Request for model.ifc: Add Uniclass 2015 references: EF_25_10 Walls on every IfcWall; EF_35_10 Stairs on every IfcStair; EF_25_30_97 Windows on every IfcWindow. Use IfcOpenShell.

First a look at what the model holds.

```python
import ifcopenshell

model = ifcopenshell.open("model.ifc")
print(model.schema)
print("classifications:", [c.Name for c in model.by_type("IfcClassification")])
for ifc_class in ("IfcDoor", "IfcRoof", "IfcStair", "IfcWall", "IfcWindow"):
    print(ifc_class, len(model.by_type(ifc_class)))
```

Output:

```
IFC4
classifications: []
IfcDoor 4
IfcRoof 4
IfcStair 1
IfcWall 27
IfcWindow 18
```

```python
import ifcopenshell
import ifcopenshell.api.classification

model = ifcopenshell.open("model.ifc")

system = ifcopenshell.api.classification.add_classification(model, classification="Uniclass 2015")

codes = {
    "IfcWall": ("EF_25_10", "Walls"),
    "IfcStair": ("EF_35_10", "Stairs"),
    "IfcWindow": ("EF_25_30_97", "Windows"),
}
for ifc_class, (code, name) in codes.items():
    products = model.by_type(ifc_class)
    ifcopenshell.api.classification.add_reference(
        model, products=products, classification=system, identification=code, name=name
    )
    print(code, len(products))

model.write("model-out.ifc")
```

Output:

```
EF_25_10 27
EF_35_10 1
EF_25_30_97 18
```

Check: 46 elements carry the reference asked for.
